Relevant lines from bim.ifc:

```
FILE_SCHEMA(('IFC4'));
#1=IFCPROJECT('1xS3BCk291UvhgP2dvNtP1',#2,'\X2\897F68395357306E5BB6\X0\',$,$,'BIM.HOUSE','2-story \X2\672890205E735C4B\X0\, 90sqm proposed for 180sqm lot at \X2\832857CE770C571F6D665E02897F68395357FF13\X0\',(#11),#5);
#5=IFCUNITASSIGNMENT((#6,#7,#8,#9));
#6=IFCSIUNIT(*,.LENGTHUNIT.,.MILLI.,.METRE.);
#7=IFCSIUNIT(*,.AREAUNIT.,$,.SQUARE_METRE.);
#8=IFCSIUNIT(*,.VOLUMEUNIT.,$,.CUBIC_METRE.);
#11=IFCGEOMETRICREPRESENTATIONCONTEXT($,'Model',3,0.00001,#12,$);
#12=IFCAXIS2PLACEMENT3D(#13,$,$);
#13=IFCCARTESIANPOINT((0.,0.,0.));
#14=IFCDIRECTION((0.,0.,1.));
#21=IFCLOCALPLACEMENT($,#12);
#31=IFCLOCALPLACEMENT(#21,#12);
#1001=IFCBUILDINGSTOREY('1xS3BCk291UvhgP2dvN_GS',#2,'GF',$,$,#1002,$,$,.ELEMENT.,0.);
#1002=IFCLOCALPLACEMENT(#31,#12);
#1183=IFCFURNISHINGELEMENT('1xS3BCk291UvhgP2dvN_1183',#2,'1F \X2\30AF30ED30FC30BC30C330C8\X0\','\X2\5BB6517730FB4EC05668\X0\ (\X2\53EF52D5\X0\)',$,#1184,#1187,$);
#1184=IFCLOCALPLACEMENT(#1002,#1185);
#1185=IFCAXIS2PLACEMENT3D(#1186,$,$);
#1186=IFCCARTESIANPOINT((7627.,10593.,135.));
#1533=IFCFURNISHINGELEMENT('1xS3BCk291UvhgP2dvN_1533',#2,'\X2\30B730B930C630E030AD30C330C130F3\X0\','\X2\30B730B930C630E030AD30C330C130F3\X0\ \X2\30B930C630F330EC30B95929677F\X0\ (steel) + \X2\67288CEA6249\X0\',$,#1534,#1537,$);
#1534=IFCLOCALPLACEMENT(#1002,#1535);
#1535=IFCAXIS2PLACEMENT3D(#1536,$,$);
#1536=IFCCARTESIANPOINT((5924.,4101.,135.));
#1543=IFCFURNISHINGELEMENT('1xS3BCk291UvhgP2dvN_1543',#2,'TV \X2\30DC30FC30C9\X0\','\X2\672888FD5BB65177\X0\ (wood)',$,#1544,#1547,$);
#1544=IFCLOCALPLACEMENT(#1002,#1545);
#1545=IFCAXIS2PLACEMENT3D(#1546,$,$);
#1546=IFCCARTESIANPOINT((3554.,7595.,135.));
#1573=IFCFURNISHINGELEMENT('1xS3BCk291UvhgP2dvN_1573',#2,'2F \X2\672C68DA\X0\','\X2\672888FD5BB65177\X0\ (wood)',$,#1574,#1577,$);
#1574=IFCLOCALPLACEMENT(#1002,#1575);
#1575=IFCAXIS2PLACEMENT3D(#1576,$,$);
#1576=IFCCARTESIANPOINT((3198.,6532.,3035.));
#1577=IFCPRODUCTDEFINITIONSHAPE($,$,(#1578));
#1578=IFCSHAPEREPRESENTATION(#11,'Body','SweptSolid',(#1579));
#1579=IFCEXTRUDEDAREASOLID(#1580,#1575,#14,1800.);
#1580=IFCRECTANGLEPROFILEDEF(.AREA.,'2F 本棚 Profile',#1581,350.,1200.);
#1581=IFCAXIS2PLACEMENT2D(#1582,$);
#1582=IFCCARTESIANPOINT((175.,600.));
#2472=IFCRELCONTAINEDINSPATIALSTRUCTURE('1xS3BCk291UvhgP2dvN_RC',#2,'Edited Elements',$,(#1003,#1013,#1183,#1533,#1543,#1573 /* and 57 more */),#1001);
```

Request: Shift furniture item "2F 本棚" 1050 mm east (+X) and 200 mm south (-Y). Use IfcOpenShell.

```python
import ifcopenshell
import ifcopenshell.api.geometry
import ifcopenshell.util.placement
import ifcopenshell.util.unit

model = ifcopenshell.open("bim.ifc")
unit_scale = ifcopenshell.util.unit.calculate_unit_scale(model)

item = model.by_id(1573)
matrix = ifcopenshell.util.placement.get_local_placement(item.ObjectPlacement)
matrix[0, 3] += 1.05 / unit_scale
matrix[1, 3] -= 0.2 / unit_scale
ifcopenshell.api.geometry.edit_object_placement(model, product=item, matrix=matrix, is_si=False)

print(ifcopenshell.util.placement.get_local_placement(item.ObjectPlacement).round(3) + 0.0)

model.write("bim_edited.ifc")
```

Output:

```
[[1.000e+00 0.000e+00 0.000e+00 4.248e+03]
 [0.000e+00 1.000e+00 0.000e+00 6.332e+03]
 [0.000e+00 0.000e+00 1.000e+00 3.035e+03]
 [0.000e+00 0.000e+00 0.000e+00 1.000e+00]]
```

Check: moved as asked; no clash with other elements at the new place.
